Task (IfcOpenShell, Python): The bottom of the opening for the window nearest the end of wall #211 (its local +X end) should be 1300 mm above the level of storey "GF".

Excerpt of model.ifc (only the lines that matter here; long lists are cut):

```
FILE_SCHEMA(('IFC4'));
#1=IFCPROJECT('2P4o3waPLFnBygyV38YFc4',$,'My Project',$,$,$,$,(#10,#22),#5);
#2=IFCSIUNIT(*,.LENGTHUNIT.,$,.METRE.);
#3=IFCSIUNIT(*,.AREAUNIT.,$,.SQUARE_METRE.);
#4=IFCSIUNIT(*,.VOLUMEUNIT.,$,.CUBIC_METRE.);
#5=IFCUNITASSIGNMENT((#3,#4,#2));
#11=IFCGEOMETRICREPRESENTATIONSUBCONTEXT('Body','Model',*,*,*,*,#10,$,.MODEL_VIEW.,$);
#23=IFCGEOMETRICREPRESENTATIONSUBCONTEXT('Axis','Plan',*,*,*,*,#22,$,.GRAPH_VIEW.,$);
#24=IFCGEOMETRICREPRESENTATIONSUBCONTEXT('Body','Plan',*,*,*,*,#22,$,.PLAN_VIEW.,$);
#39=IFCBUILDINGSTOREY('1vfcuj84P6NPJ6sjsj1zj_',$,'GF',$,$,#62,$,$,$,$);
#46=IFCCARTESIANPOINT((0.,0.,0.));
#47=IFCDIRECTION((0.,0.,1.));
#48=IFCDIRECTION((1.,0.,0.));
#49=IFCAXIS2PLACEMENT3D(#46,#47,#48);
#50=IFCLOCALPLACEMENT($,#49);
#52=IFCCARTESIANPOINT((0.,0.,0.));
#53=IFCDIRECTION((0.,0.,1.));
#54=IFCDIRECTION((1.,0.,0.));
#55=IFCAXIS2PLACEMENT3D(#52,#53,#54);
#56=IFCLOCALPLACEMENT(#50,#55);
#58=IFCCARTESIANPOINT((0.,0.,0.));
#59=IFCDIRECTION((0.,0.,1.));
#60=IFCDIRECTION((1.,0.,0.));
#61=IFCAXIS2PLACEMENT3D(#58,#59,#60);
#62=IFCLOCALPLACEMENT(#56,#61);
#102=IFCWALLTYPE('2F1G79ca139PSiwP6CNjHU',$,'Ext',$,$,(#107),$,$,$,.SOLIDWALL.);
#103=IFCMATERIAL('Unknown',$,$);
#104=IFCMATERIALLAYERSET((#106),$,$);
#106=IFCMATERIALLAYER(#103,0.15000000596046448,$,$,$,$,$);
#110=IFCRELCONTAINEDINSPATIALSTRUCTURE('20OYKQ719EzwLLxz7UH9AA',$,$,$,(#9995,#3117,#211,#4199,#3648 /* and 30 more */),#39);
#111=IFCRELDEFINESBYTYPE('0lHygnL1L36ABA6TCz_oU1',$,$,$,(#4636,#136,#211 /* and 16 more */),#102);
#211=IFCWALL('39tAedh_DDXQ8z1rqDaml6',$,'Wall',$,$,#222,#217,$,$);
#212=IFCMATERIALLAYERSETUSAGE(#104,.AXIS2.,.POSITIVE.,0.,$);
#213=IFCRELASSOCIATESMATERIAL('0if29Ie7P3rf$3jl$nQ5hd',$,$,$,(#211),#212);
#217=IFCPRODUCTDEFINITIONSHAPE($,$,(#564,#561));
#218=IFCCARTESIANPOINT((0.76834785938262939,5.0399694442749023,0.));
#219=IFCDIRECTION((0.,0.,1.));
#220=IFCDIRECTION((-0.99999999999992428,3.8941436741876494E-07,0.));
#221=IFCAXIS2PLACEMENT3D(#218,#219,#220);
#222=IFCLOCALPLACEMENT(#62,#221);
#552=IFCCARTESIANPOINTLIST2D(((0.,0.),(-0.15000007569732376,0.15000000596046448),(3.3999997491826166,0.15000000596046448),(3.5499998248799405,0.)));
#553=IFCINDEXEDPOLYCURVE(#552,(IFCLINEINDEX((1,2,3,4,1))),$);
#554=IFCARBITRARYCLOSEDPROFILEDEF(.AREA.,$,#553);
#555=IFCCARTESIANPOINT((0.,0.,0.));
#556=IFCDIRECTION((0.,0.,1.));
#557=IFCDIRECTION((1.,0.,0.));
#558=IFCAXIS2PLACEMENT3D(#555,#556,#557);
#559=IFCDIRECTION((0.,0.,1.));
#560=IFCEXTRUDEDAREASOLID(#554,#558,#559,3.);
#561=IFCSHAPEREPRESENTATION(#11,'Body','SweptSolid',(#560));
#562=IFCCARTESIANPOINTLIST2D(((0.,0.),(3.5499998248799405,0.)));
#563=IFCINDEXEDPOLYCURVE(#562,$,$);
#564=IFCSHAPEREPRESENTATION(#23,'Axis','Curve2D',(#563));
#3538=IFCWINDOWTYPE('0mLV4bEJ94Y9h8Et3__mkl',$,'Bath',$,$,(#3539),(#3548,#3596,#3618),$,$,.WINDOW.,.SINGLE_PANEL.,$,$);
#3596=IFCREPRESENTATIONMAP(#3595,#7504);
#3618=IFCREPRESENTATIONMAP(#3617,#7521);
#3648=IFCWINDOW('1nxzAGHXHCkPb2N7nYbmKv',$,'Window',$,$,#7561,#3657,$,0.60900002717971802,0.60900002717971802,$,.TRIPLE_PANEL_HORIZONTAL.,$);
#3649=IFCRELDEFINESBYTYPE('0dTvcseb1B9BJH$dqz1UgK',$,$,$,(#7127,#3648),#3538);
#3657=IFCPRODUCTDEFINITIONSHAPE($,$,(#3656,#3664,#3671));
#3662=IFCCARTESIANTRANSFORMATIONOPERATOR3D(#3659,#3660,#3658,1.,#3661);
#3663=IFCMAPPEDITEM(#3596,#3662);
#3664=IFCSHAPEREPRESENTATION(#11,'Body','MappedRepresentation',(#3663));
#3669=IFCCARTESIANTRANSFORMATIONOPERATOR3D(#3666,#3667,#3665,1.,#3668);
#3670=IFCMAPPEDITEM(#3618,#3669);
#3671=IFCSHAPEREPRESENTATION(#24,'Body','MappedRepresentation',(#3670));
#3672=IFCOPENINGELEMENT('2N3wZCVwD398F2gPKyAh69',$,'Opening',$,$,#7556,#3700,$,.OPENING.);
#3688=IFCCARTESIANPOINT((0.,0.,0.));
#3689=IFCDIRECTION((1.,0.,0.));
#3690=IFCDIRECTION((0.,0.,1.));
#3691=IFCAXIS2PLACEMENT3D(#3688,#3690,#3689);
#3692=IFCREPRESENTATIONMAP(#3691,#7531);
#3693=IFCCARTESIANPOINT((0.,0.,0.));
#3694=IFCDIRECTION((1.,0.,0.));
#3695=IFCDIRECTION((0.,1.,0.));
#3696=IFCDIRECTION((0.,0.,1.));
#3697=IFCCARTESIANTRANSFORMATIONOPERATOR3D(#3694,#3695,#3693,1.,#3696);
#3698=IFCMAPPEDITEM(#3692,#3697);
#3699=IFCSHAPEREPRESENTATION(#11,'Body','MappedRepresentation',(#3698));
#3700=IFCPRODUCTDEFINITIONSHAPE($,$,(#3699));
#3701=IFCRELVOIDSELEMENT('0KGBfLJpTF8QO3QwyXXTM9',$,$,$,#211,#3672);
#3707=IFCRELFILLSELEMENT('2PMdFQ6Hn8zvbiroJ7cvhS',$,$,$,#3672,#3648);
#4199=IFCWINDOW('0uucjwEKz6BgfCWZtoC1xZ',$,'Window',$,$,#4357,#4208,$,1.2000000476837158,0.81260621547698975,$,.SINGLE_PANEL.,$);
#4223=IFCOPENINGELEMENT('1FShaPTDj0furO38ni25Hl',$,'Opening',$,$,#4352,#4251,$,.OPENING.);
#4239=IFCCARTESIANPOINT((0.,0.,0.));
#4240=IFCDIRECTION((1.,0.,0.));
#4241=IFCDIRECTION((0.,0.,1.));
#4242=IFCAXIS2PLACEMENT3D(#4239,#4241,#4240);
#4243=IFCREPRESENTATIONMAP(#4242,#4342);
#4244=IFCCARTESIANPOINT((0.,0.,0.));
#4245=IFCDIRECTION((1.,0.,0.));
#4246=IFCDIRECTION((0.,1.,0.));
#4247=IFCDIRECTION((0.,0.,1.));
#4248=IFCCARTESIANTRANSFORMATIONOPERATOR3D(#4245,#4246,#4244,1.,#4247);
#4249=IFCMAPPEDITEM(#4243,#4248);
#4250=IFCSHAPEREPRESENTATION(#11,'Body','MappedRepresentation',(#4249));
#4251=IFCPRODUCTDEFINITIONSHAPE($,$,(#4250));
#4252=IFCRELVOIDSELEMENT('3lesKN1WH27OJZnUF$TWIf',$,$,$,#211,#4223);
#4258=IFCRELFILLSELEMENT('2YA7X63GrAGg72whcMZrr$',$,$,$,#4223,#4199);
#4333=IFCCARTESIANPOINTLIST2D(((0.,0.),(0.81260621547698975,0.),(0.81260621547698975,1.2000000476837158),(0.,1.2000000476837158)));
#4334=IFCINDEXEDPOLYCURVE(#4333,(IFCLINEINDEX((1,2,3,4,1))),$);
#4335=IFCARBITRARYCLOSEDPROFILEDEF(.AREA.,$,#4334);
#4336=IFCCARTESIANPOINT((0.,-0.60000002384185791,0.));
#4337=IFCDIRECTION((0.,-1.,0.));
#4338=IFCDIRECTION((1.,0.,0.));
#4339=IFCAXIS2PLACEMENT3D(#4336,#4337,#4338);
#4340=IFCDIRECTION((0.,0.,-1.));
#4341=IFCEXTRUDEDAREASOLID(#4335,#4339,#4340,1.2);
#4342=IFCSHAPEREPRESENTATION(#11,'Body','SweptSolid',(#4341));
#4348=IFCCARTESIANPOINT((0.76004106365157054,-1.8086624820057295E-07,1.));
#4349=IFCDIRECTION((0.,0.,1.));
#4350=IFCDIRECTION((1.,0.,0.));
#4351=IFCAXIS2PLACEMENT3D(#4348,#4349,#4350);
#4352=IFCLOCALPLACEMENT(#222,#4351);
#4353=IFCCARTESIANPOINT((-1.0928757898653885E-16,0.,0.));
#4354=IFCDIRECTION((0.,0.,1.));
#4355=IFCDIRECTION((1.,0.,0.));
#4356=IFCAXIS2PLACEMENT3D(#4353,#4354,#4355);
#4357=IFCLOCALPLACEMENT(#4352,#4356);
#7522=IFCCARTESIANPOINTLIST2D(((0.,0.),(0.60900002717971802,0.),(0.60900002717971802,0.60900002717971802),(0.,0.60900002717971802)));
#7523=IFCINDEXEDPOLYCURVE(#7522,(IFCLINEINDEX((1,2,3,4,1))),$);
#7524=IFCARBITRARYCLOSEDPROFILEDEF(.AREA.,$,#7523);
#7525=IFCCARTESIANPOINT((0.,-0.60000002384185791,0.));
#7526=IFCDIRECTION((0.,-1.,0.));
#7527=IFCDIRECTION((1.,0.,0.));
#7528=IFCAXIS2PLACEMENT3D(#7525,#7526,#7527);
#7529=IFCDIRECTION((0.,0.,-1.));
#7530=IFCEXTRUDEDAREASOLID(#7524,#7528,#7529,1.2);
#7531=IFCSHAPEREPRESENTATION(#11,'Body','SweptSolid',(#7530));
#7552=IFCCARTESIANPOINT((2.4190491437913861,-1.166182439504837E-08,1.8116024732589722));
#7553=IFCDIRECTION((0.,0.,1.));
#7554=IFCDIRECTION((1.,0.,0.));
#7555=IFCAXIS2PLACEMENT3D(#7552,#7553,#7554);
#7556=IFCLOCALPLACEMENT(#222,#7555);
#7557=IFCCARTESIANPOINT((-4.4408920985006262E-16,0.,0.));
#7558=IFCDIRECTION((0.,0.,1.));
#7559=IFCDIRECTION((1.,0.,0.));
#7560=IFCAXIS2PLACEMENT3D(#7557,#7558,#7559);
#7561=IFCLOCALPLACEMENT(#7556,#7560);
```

```python
import numpy as np
import ifcopenshell
import ifcopenshell.api.geometry
import ifcopenshell.geom
import ifcopenshell.util.element
import ifcopenshell.util.placement
import ifcopenshell.util.shape
import ifcopenshell.util.unit

model = ifcopenshell.open("model.ifc")
unit_scale = ifcopenshell.util.unit.calculate_unit_scale(model)

window = model.by_guid("1nxzAGHXHCkPb2N7nYbmKv")
opening = window.FillsVoids[0].RelatingOpeningElement
storey = ifcopenshell.util.element.get_container(window, ifc_class="IfcBuildingStorey")
level = ifcopenshell.util.placement.get_local_placement(storey.ObjectPlacement)[2, 3]

# The opening's origin need not be at the sill, so measure its lowest point.
shape = ifcopenshell.geom.create_shape(ifcopenshell.geom.settings(), opening)
bottom = ifcopenshell.util.shape.get_shape_bottom_elevation(shape, shape.geometry) / unit_scale
dz = level + 1.3 / unit_scale - bottom

shift = np.array([0.0, 0.0, dz])
# The window is placed relative to its opening, so it follows when the opening moves.
matrix = ifcopenshell.util.placement.get_local_placement(opening.ObjectPlacement)
matrix[:3, 3] += shift
ifcopenshell.api.geometry.edit_object_placement(
    model, product=opening, matrix=matrix, is_si=False, should_transform_children=True
)

print(f"moved by {dz * unit_scale:+.3f} m")

model.write("model_edited.ifc")
```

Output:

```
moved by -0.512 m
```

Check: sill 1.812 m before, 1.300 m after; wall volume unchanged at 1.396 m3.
